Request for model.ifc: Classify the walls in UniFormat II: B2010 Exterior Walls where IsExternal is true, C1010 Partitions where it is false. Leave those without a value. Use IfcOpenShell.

First a look at what the model holds.

```python
import ifcopenshell
import ifcopenshell.util.element

model = ifcopenshell.open("model.ifc")
print(model.schema)
print("classifications:", [c.Name for c in model.by_type("IfcClassification")])
values = [ifcopenshell.util.element.get_pset(e, "Pset_WallCommon", "IsExternal") for e in model.by_type("IfcWall")]
for value in (True, False, None):
    print("IsExternal", value, values.count(value))
```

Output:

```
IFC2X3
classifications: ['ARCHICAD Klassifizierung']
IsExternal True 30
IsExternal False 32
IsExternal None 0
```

```python
import ifcopenshell
import ifcopenshell.api.classification
import ifcopenshell.util.element

model = ifcopenshell.open("model.ifc")

# IFC2X3 requires Source and Edition and has no link from the project to the system.
system = model.create_entity("IfcClassification", Source="ASTM", Edition="E1557", Name="UniFormat II")

walls = model.by_type("IfcWall")
external = {e: ifcopenshell.util.element.get_pset(e, "Pset_WallCommon", "IsExternal") for e in walls}
for flag, code, name in ((True, "B2010", "Exterior Walls"), (False, "C1010", "Partitions")):
    products = [e for e in walls if external[e] is flag]
    ifcopenshell.api.classification.add_reference(
        model, products=products, classification=system, identification=code, name=name
    )
    print(code, len(products))

model.write("model_v2.ifc")
```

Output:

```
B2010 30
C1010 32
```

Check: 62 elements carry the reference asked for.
